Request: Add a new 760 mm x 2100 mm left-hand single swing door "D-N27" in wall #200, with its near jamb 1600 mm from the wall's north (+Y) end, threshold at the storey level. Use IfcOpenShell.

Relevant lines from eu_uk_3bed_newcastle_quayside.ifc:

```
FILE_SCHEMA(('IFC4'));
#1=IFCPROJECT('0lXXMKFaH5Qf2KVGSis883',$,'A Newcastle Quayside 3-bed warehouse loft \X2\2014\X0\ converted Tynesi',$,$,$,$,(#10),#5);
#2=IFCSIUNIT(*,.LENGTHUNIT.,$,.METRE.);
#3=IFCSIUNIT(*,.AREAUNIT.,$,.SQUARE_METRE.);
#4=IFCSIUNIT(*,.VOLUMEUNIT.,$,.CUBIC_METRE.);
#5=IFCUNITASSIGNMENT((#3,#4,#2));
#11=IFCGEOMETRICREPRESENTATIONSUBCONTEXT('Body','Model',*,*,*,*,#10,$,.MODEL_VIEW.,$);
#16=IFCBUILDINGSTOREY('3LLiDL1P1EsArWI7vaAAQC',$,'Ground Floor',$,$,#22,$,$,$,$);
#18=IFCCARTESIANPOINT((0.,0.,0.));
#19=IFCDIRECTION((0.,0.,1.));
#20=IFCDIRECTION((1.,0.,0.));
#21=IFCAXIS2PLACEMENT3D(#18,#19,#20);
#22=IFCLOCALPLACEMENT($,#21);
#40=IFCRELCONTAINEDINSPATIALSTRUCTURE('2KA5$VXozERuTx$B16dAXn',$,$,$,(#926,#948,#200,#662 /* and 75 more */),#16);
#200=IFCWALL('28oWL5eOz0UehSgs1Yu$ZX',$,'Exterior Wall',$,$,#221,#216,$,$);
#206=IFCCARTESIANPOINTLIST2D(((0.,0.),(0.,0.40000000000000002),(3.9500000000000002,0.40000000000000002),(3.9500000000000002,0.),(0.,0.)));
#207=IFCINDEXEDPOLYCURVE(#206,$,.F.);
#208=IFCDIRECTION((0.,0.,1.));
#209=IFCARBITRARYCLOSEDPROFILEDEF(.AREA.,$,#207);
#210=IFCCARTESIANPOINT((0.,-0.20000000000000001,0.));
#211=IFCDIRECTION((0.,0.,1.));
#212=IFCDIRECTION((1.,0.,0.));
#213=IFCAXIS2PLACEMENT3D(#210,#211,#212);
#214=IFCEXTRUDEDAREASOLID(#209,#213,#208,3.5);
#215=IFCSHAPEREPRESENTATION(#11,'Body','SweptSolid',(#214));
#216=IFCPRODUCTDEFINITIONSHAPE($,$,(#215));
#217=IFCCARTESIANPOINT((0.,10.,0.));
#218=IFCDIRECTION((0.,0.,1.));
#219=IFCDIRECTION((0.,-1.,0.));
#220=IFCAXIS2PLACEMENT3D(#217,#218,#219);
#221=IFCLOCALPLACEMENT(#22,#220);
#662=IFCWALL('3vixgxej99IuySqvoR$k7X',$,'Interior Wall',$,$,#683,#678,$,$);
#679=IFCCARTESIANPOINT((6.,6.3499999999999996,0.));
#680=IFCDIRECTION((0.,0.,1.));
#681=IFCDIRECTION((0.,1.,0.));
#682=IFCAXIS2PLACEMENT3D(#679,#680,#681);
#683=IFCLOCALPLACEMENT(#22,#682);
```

```python
import numpy as np
import ifcopenshell
import ifcopenshell.api.feature
import ifcopenshell.api.geometry
import ifcopenshell.api.root
import ifcopenshell.api.spatial
import ifcopenshell.geom
import ifcopenshell.util.element
import ifcopenshell.util.placement
import ifcopenshell.util.representation
import ifcopenshell.util.shape
import ifcopenshell.util.unit

model = ifcopenshell.open("eu_uk_3bed_newcastle_quayside.ifc")
unit_scale = ifcopenshell.util.unit.calculate_unit_scale(model)
settings = ifcopenshell.geom.settings()


def volume(element):
    """Net volume in cubic metres, openings subtracted."""
    shape = ifcopenshell.geom.create_shape(settings, element)
    return ifcopenshell.util.shape.get_volume(shape.geometry)


wall = model.by_guid("28oWL5eOz0UehSgs1Yu$ZX")
storey = ifcopenshell.util.element.get_container(wall, ifc_class="IfcBuildingStorey")
context = ifcopenshell.util.representation.get_context(model, "Model", "Body", "MODEL_VIEW")
before = volume(wall)

width, height, from_end, sill = 0.76, 2.1, 1.6, 0.0  # metres

# The wall runs along its own X axis, and the end named is its -X end.
wall_shape = ifcopenshell.geom.create_shape(settings, wall)
x, y, z = ifcopenshell.util.shape.get_vertices(wall_shape.geometry).T
start = x.min() + from_end
face, thickness = float(y.min()), float(y.max() - y.min())
wall_matrix = ifcopenshell.util.placement.get_local_placement(wall.ObjectPlacement)
level = ifcopenshell.util.placement.get_local_placement(storey.ObjectPlacement)[2, 3]


def in_wall(x, y):
    """Placement at x, y metres in the wall's axes, at sill height."""
    matrix = wall_matrix.copy()
    matrix[:, 3] = wall_matrix @ np.array([x / unit_scale, y / unit_scale, 0.0, 1.0])
    matrix[2, 3] = level + sill / unit_scale
    return matrix


# Opening: a box that overshoots both wall faces by 50 mm.
opening = ifcopenshell.api.root.create_entity(model, ifc_class="IfcOpeningElement", predefined_type="OPENING")
box = ifcopenshell.api.geometry.add_wall_representation(
    model, context=context, length=width, height=height, thickness=thickness + 0.1
)
ifcopenshell.api.geometry.assign_representation(model, product=opening, representation=box)
ifcopenshell.api.geometry.edit_object_placement(model, product=opening, matrix=in_wall(start, face - 0.05), is_si=False)
ifcopenshell.api.feature.add_feature(model, feature=opening, element=wall)

door = ifcopenshell.api.root.create_entity(model, ifc_class="IfcDoor", name="D-N27", predefined_type="DOOR")
door.OverallWidth, door.OverallHeight = width / unit_scale, height / unit_scale
door.OperationType = "SINGLE_SWING_LEFT"
body = ifcopenshell.api.geometry.add_door_representation(
    model,
    context=context,
    overall_width=door.OverallWidth,
    overall_height=door.OverallHeight,
    operation_type="SINGLE_SWING_LEFT",
    lining_properties={"LiningDepth": thickness / unit_scale, "ThresholdDepth": thickness / unit_scale},
)
ifcopenshell.api.geometry.assign_representation(model, product=door, representation=body)
ifcopenshell.api.spatial.assign_container(model, products=[door], relating_structure=storey)
ifcopenshell.api.feature.add_filling(model, opening=opening, element=door)

# The lining spans the wall, so the door starts at the wall face.
ifcopenshell.api.geometry.edit_object_placement(model, product=door, matrix=in_wall(start, face), is_si=False)

after = volume(wall)

print(f"wall volume {before:.3f} -> {after:.3f} m3")

model.write("eu_uk_3bed_newcastle_quayside_updated.ifc")
```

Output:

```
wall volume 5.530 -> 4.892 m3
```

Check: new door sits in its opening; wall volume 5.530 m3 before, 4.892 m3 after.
